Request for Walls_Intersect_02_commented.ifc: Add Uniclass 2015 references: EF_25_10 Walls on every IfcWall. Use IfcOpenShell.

First a look at what the model holds.

```python
import ifcopenshell

model = ifcopenshell.open("Walls_Intersect_02_commented.ifc")
print(model.schema)
print("classifications:", [c.Name for c in model.by_type("IfcClassification")])
for ifc_class in ("IfcDoor", "IfcRoof", "IfcStair", "IfcWall", "IfcWindow"):
    print(ifc_class, len(model.by_type(ifc_class)))
```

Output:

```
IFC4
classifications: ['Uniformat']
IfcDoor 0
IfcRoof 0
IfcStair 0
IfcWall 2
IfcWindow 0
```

```python
import ifcopenshell
import ifcopenshell.api.classification

model = ifcopenshell.open("Walls_Intersect_02_commented.ifc")

system = ifcopenshell.api.classification.add_classification(model, classification="Uniclass 2015")

codes = {
    "IfcWall": ("EF_25_10", "Walls"),
}
for ifc_class, (code, name) in codes.items():
    products = model.by_type(ifc_class)
    ifcopenshell.api.classification.add_reference(
        model, products=products, classification=system, identification=code, name=name
    )
    print(code, len(products))

model.write("Walls_Intersect_02_commented_v2.ifc")
```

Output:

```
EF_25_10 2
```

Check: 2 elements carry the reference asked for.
